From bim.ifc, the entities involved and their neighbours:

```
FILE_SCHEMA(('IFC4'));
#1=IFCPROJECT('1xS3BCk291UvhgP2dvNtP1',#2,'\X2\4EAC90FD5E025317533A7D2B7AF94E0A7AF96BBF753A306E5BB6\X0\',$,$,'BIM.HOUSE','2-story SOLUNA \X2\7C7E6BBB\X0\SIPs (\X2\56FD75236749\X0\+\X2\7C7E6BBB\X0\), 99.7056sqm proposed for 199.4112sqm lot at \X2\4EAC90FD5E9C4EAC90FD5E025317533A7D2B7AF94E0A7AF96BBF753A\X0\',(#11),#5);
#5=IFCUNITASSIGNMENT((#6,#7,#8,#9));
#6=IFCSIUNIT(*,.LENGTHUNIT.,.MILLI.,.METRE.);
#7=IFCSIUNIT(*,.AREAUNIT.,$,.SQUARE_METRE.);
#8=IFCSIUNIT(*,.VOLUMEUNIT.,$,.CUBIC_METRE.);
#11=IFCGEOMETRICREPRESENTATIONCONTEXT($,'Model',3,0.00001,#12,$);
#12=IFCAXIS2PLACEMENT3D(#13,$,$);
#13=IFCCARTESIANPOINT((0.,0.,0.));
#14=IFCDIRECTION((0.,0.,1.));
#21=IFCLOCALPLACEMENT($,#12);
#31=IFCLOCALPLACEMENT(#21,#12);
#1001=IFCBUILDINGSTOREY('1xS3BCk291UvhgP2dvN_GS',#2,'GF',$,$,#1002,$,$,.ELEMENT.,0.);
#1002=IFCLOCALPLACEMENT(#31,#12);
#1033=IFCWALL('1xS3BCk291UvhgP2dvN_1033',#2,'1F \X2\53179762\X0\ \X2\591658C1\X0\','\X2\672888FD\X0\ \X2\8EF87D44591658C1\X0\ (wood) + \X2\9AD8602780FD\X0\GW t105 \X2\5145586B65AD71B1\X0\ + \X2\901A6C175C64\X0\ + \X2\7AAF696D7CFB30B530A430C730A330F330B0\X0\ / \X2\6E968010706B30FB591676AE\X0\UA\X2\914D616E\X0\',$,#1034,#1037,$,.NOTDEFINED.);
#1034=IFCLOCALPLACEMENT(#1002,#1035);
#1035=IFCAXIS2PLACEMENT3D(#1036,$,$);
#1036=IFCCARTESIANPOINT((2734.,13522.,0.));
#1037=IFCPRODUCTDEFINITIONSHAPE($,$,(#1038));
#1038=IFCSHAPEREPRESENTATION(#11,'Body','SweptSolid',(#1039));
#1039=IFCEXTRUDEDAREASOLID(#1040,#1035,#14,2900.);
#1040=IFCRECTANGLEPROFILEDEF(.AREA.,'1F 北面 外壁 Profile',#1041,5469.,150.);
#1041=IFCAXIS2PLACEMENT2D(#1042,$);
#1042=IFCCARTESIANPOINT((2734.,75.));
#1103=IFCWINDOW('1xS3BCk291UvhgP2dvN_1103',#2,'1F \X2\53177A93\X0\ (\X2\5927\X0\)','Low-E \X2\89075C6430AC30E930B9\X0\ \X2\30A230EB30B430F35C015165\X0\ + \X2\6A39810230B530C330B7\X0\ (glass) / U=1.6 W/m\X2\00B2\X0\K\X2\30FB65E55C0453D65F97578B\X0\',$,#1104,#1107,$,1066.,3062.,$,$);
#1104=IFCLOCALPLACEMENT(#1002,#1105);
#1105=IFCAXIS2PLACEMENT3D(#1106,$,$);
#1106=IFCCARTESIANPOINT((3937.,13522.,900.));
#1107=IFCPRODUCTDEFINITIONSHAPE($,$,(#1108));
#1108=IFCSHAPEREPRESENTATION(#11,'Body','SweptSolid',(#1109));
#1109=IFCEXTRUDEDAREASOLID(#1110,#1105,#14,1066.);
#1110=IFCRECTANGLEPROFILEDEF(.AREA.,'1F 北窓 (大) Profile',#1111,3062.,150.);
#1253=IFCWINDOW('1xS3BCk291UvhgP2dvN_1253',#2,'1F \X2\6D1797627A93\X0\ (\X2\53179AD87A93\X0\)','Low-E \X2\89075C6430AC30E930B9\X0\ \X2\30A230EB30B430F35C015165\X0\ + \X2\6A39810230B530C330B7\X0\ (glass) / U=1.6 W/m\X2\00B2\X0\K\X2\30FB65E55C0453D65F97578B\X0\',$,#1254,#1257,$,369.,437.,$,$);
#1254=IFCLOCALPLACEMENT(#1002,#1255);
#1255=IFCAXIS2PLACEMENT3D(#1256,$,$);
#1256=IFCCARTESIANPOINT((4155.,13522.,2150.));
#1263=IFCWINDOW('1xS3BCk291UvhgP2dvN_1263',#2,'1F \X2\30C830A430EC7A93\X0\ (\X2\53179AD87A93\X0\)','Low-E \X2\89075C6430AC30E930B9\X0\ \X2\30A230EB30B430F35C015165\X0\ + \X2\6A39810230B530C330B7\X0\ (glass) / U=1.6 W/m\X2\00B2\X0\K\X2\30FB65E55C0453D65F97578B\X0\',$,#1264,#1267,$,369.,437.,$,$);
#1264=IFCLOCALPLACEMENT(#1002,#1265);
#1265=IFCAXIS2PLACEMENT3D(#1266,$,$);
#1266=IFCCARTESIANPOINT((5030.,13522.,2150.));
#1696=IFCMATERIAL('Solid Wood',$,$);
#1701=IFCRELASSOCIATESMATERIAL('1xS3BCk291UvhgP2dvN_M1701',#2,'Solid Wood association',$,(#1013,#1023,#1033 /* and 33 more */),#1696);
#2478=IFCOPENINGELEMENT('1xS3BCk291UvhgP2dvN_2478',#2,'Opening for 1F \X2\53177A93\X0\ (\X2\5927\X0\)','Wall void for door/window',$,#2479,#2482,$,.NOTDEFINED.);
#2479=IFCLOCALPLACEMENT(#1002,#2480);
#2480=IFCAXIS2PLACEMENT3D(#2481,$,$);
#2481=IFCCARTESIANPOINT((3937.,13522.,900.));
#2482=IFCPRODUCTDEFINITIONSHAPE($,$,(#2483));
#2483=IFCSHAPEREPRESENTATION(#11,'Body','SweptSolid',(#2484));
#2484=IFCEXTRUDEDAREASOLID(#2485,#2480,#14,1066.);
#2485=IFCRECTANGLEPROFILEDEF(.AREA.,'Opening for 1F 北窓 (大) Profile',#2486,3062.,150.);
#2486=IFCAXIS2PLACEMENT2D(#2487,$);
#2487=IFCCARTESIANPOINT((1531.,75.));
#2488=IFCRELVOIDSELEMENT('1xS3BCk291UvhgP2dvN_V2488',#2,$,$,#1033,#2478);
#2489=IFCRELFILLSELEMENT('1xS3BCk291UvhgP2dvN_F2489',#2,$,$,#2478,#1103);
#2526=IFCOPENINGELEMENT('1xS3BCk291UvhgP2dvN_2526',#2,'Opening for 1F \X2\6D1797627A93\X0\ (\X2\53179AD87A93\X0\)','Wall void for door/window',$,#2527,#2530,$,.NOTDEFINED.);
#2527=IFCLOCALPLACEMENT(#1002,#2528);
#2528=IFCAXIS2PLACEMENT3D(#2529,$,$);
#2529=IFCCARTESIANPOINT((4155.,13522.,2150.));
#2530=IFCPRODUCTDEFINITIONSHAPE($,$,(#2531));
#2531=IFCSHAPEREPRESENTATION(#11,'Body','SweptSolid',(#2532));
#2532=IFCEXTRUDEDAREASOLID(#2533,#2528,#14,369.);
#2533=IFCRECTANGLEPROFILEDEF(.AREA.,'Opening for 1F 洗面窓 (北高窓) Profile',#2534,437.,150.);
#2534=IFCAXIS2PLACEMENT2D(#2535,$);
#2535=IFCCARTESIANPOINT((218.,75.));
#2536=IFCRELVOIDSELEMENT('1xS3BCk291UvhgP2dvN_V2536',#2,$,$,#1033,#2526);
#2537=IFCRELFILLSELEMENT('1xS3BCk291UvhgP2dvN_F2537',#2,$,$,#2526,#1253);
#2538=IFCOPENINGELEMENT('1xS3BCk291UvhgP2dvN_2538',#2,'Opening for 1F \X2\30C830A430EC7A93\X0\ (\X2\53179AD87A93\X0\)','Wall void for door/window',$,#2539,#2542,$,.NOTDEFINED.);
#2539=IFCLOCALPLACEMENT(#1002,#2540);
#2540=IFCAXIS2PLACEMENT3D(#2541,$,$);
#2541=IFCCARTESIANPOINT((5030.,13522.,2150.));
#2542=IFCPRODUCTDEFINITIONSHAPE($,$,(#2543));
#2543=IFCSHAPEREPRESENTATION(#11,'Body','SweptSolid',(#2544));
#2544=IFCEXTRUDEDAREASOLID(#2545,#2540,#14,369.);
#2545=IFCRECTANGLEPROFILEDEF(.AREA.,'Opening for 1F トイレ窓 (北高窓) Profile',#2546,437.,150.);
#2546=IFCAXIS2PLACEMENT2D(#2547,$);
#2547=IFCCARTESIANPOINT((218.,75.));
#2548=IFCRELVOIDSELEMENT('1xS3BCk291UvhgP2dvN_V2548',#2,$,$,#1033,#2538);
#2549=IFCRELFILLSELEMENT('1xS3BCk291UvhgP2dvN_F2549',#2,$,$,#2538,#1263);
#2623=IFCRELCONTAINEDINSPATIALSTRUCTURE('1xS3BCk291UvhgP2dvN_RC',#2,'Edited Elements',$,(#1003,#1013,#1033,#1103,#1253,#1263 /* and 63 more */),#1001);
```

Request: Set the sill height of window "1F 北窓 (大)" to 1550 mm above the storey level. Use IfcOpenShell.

```python
import numpy as np
import ifcopenshell
import ifcopenshell.api.geometry
import ifcopenshell.geom
import ifcopenshell.util.element
import ifcopenshell.util.placement
import ifcopenshell.util.shape
import ifcopenshell.util.unit

model = ifcopenshell.open("bim.ifc")
unit_scale = ifcopenshell.util.unit.calculate_unit_scale(model)

window = model.by_id(1103)
opening = window.FillsVoids[0].RelatingOpeningElement
storey = ifcopenshell.util.element.get_container(window, ifc_class="IfcBuildingStorey")
level = ifcopenshell.util.placement.get_local_placement(storey.ObjectPlacement)[2, 3]

# The opening's origin need not be at the sill, so measure its lowest point.
shape = ifcopenshell.geom.create_shape(ifcopenshell.geom.settings(), opening)
bottom = ifcopenshell.util.shape.get_shape_bottom_elevation(shape, shape.geometry) / unit_scale
dz = level + 1550.0 - bottom

shift = np.array([0.0, 0.0, dz])
# The window is not placed relative to its opening, so move both.
for product in (opening, window):
    matrix = ifcopenshell.util.placement.get_local_placement(product.ObjectPlacement)
    matrix[:3, 3] += shift
    ifcopenshell.api.geometry.edit_object_placement(model, product=product, matrix=matrix, is_si=False)

print(f"moved by {dz * unit_scale:+.3f} m")

model.write("bim_edited.ifc")
```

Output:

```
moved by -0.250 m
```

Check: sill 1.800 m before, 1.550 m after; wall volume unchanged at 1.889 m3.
